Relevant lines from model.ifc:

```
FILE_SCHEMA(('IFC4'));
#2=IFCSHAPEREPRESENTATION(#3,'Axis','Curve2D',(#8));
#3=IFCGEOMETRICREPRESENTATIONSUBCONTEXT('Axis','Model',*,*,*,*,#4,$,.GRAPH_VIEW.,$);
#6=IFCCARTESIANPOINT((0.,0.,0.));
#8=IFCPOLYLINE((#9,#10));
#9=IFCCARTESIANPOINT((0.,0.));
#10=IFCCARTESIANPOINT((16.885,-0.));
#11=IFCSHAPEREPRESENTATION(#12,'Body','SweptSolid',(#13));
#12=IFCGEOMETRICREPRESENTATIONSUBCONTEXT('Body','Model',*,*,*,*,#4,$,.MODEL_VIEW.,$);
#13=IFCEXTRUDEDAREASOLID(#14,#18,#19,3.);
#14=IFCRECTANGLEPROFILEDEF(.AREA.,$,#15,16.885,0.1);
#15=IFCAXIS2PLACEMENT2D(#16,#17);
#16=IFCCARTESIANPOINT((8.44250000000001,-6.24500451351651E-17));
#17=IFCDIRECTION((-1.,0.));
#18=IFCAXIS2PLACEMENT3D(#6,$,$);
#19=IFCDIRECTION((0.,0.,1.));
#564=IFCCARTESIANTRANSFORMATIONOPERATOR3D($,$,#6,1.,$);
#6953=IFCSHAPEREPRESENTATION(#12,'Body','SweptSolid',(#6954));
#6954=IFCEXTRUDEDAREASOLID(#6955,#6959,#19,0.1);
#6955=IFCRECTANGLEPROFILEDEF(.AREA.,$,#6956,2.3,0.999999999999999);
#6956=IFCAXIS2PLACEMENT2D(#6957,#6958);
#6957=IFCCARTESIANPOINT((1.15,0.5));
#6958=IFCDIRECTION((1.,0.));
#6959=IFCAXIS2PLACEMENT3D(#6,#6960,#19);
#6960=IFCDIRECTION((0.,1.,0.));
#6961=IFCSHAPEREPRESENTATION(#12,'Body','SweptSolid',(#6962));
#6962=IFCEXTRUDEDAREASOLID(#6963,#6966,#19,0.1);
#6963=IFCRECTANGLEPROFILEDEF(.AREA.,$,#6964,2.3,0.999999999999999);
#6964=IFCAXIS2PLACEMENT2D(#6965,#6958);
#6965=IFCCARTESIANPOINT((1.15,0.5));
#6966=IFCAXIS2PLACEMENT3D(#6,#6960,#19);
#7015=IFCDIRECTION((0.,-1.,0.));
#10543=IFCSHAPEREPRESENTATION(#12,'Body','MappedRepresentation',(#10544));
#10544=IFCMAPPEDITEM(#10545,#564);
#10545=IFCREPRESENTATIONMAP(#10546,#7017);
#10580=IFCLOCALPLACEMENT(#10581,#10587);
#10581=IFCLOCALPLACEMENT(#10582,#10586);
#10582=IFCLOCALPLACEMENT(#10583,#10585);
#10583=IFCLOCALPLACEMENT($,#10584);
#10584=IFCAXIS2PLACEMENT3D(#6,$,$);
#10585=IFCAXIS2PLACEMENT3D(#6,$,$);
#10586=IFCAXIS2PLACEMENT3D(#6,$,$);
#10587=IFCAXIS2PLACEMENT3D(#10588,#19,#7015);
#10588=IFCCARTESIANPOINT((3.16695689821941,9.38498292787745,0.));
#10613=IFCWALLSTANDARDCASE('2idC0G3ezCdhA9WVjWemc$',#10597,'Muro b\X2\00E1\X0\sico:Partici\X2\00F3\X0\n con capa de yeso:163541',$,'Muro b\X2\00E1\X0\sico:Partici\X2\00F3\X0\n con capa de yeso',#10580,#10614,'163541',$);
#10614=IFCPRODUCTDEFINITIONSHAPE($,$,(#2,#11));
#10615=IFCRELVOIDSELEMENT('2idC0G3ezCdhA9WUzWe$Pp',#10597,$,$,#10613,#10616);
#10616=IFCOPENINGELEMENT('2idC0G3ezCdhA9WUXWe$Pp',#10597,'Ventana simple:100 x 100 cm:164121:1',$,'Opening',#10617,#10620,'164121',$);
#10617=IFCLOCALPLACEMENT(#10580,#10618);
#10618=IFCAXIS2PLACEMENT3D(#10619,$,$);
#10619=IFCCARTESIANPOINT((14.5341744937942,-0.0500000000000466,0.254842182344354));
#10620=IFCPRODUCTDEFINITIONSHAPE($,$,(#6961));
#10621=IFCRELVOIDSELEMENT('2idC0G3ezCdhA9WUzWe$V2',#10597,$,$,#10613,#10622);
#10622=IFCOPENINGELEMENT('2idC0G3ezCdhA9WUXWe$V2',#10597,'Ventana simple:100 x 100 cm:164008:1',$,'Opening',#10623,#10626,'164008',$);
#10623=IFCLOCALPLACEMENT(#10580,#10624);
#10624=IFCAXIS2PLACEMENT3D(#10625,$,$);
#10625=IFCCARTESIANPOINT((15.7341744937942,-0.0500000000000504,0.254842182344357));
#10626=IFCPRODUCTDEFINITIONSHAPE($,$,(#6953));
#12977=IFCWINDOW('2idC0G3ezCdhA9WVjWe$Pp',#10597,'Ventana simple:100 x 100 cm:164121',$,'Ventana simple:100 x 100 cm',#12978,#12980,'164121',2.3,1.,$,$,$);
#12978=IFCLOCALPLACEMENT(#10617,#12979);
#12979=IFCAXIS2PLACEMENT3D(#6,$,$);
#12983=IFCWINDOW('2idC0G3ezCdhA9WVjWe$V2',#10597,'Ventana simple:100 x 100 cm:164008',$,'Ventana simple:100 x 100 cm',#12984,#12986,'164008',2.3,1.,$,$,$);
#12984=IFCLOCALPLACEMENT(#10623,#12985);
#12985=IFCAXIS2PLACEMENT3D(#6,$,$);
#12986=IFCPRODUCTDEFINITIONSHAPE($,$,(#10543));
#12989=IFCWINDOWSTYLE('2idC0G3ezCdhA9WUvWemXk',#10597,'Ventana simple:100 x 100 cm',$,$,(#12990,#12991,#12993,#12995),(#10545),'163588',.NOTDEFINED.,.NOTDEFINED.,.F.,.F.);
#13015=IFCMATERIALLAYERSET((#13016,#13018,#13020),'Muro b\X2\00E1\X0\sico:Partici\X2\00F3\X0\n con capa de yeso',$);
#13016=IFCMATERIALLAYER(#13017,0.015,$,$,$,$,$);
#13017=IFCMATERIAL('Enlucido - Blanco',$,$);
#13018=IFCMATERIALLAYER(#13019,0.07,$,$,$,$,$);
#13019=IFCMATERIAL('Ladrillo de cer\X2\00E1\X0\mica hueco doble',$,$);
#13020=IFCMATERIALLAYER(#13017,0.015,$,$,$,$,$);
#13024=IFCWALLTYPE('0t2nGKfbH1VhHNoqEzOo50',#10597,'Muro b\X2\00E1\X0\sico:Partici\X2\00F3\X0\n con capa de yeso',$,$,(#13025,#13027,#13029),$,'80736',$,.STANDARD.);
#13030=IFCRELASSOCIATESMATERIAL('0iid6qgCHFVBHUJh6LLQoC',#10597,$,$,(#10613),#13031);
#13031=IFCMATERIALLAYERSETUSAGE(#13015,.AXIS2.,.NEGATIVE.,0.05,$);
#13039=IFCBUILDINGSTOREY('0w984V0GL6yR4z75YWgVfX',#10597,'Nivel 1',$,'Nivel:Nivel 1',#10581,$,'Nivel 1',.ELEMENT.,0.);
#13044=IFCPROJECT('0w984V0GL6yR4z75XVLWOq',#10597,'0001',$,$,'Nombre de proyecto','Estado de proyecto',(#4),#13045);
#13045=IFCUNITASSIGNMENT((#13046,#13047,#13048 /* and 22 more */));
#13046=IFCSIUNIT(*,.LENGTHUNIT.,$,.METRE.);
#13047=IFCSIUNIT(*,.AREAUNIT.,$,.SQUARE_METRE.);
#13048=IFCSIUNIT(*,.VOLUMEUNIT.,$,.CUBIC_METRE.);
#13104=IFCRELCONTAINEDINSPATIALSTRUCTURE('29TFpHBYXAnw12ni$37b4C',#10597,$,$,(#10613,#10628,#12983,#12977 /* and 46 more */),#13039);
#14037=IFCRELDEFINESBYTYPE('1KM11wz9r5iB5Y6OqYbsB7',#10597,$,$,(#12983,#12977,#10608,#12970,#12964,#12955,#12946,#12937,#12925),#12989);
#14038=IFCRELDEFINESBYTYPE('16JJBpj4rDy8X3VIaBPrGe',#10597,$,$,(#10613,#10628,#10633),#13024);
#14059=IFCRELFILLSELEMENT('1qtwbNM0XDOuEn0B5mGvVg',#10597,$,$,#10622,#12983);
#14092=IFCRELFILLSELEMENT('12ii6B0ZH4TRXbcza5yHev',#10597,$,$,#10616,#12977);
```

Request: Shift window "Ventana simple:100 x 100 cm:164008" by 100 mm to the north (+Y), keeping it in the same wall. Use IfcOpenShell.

```python
import ifcopenshell
import ifcopenshell.api.geometry
import ifcopenshell.util.placement
import ifcopenshell.util.unit

model = ifcopenshell.open("model.ifc")
unit_scale = ifcopenshell.util.unit.calculate_unit_scale(model)

window = model.by_id(12983)
opening = window.FillsVoids[0].RelatingOpeningElement
wall = opening.VoidsElements[0].RelatingBuildingElement

wall_matrix = ifcopenshell.util.placement.get_local_placement(wall.ObjectPlacement)
shift = wall_matrix[:3, 0] * -0.1 / unit_scale
before = ifcopenshell.util.placement.get_local_placement(window.ObjectPlacement)[:3, 3].copy()

# The window is placed relative to its opening, so it follows when the opening moves.
matrix = ifcopenshell.util.placement.get_local_placement(opening.ObjectPlacement)
matrix[:3, 3] += shift
ifcopenshell.api.geometry.edit_object_placement(
    model, product=opening, matrix=matrix, is_si=False, should_transform_children=True
)

after = ifcopenshell.util.placement.get_local_placement(window.ObjectPlacement)[:3, 3]
print("window moved by", (after - before).round(3) + 0.0)

model.write("model_rev.ifc")
```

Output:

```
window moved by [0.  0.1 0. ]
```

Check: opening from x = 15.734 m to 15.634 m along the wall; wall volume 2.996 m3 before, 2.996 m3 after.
